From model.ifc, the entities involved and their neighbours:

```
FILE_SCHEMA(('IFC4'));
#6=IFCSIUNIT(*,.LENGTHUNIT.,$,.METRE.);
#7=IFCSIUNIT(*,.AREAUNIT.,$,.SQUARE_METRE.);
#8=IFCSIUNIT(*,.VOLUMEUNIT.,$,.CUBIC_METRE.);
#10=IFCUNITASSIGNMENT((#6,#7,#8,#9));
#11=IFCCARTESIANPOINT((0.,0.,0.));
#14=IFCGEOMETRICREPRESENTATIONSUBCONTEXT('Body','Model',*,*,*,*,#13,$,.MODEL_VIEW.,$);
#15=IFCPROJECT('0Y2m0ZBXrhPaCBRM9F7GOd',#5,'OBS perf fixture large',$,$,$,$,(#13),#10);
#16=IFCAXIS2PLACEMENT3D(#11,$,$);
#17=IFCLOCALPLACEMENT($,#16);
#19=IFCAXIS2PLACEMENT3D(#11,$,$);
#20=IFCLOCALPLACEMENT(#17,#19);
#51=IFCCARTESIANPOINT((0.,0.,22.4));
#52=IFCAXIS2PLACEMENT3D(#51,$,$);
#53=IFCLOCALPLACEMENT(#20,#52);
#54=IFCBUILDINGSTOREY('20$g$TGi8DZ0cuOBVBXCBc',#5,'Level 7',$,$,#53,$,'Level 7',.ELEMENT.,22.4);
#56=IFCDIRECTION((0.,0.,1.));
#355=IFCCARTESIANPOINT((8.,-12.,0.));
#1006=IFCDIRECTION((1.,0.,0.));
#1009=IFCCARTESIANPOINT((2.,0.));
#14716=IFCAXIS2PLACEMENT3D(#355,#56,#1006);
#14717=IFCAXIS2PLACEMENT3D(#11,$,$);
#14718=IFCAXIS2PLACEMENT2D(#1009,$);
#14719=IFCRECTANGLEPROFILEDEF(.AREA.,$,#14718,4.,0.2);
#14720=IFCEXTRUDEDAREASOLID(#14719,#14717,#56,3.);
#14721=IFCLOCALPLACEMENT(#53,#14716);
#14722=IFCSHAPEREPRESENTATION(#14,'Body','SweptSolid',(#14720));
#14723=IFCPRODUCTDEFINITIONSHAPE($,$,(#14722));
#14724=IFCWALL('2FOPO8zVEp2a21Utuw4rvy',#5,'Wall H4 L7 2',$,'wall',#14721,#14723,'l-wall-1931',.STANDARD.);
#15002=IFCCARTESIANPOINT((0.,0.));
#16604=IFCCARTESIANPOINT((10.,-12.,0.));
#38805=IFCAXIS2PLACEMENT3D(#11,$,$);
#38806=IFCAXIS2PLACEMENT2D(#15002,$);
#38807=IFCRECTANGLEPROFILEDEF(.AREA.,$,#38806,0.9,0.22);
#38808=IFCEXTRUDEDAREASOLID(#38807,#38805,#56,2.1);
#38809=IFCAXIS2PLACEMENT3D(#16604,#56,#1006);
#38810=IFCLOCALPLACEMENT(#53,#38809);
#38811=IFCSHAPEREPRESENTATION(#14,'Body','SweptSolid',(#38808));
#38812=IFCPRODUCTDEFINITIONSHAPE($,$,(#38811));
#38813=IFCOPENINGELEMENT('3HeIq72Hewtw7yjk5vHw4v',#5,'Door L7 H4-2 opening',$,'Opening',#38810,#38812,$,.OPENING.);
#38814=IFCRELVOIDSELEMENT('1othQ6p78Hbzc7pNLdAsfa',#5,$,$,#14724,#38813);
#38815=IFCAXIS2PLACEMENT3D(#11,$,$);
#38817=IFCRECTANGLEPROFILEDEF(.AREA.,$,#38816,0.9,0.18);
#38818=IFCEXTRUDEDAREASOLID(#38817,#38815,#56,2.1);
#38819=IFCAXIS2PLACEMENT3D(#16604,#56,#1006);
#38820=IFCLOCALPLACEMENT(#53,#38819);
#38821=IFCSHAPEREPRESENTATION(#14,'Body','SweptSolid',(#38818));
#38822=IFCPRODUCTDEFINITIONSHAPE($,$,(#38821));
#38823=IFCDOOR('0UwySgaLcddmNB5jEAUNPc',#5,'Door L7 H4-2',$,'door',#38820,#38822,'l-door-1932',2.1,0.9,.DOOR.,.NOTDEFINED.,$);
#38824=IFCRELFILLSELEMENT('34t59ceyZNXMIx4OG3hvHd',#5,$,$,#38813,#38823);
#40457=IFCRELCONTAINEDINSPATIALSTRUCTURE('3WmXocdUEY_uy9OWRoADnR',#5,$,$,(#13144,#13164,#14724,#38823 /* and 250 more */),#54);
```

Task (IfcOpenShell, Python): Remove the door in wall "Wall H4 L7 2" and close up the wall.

```python
import ifcopenshell
import ifcopenshell.api.feature
import ifcopenshell.api.root
import ifcopenshell.geom
import ifcopenshell.util.shape

model = ifcopenshell.open("model.ifc")
settings = ifcopenshell.geom.settings()


def volume(element):
    """Net volume in cubic metres, openings subtracted."""
    shape = ifcopenshell.geom.create_shape(settings, element)
    return ifcopenshell.util.shape.get_volume(shape.geometry)


door = model.by_guid("0UwySgaLcddmNB5jEAUNPc")
opening = door.FillsVoids[0].RelatingOpeningElement
wall = opening.VoidsElements[0].RelatingBuildingElement
before = volume(wall)

ifcopenshell.api.root.remove_product(model, product=door)
ifcopenshell.api.feature.remove_feature(model, feature=opening)

after = volume(wall)

print(f"wall volume {before:.3f} -> {after:.3f} m3")

model.write("model_rev.ifc")
```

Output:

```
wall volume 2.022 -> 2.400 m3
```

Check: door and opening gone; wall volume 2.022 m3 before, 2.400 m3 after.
